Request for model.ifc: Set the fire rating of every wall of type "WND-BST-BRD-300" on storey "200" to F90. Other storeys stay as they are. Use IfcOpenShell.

First a look at what the model holds.

```python
import ifcopenshell
import ifcopenshell.util.element

model = ifcopenshell.open("model.ifc")
print(model.schema)
storey = next(s for s in model.by_type("IfcBuildingStorey") if s.Name == "200")
walls = [e for e in ifcopenshell.util.element.get_decomposition(storey) if e.is_a("IfcWall")]
seen = {}
for e in walls:
    element_type = ifcopenshell.util.element.get_type(e)
    key = (element_type.Name if element_type != e and element_type else None, ifcopenshell.util.element.get_pset(e, "Pset_WallCommon", "FireRating"))
    seen[key] = seen.get(key, 0) + 1
for (name, value), count in sorted(seen.items(), key=str):
    print(count, "x", name, "|", value)
```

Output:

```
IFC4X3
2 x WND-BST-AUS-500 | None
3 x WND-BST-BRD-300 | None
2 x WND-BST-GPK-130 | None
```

```python
import ifcopenshell
import ifcopenshell.api.pset
import ifcopenshell.util.element

model = ifcopenshell.open("model.ifc")

storey = next(s for s in model.by_type("IfcBuildingStorey") if s.Name == "200")
walls = [e for e in ifcopenshell.util.element.get_decomposition(storey) if e.is_a("IfcWall")]

count = 0
for e in walls:
    element_type = ifcopenshell.util.element.get_type(e)
    if element_type in (None, e) or element_type.Name != "WND-BST-BRD-300":
        continue
    # add_pset returns the element's existing set when there is one.
    pset = ifcopenshell.api.pset.add_pset(model, product=e, name="Pset_WallCommon")
    ifcopenshell.api.pset.edit_pset(model, pset=pset, properties={"FireRating": "F90"})
    count += 1

print(count, "walls updated")

model.write("model_v2.ifc")
```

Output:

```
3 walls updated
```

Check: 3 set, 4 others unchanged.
